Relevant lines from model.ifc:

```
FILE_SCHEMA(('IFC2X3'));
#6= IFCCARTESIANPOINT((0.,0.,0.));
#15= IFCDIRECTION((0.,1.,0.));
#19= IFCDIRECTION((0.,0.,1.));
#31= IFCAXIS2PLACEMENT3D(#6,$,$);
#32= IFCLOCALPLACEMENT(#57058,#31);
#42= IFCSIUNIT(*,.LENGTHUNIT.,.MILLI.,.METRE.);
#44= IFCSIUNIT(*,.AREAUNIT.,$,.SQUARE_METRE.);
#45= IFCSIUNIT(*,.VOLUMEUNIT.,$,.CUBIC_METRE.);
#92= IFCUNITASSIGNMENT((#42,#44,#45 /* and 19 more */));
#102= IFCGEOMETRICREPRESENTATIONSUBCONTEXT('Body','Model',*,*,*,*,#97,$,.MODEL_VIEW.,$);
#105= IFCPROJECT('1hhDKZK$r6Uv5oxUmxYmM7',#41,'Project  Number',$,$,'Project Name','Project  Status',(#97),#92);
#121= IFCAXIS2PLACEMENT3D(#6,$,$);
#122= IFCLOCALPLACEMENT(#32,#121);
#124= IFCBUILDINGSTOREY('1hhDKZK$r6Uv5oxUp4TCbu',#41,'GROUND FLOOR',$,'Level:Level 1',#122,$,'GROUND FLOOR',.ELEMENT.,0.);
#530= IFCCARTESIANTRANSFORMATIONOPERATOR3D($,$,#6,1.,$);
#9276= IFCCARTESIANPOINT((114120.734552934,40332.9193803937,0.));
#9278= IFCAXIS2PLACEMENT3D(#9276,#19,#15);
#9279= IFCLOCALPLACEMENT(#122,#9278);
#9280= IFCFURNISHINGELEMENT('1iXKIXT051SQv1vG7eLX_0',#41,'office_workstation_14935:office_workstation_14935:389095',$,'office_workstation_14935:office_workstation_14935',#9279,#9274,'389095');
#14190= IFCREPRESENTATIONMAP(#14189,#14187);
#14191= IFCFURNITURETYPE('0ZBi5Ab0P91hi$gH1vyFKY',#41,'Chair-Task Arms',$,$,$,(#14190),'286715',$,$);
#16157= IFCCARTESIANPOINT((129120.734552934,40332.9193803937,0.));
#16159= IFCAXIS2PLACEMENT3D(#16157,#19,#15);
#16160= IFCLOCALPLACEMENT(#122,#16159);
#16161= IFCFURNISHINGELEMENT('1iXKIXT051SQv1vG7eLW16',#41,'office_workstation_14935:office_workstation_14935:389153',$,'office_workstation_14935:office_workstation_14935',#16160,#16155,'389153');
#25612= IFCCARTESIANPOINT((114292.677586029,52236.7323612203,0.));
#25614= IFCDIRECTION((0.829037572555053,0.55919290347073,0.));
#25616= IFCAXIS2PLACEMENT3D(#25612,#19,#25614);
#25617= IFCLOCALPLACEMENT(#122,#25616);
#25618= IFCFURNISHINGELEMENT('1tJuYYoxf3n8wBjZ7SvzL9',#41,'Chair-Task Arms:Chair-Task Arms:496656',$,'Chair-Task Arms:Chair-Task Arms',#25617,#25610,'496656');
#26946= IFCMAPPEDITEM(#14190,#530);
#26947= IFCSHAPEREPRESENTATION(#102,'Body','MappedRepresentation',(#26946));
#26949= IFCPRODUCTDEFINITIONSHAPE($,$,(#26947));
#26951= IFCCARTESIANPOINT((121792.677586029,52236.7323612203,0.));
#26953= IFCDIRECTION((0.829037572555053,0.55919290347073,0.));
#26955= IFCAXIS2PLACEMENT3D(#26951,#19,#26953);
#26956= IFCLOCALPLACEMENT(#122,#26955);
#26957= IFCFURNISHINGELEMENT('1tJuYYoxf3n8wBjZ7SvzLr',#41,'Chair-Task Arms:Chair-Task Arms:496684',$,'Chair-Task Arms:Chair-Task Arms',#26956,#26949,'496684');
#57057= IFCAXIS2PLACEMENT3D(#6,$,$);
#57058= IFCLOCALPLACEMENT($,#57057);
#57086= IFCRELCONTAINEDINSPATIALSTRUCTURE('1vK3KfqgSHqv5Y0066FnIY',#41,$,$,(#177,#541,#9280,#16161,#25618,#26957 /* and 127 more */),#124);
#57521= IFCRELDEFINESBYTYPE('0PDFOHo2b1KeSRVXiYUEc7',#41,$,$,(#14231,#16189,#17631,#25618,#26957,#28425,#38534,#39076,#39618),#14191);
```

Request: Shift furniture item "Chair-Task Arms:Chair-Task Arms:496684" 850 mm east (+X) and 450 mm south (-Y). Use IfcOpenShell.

```python
import ifcopenshell
import ifcopenshell.api.geometry
import ifcopenshell.util.placement
import ifcopenshell.util.unit

model = ifcopenshell.open("model.ifc")
unit_scale = ifcopenshell.util.unit.calculate_unit_scale(model)

item = model.by_id(26957)
matrix = ifcopenshell.util.placement.get_local_placement(item.ObjectPlacement)
matrix[0, 3] += 0.85 / unit_scale
matrix[1, 3] -= 0.45 / unit_scale
ifcopenshell.api.geometry.edit_object_placement(model, product=item, matrix=matrix, is_si=False)

print(ifcopenshell.util.placement.get_local_placement(item.ObjectPlacement).round(3) + 0.0)

model.write("model_edited.ifc")
```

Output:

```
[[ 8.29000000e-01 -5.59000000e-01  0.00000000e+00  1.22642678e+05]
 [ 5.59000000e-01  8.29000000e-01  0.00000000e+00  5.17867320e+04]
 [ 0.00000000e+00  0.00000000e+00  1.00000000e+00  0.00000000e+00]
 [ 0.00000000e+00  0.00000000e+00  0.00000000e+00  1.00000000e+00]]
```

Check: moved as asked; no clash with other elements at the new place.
